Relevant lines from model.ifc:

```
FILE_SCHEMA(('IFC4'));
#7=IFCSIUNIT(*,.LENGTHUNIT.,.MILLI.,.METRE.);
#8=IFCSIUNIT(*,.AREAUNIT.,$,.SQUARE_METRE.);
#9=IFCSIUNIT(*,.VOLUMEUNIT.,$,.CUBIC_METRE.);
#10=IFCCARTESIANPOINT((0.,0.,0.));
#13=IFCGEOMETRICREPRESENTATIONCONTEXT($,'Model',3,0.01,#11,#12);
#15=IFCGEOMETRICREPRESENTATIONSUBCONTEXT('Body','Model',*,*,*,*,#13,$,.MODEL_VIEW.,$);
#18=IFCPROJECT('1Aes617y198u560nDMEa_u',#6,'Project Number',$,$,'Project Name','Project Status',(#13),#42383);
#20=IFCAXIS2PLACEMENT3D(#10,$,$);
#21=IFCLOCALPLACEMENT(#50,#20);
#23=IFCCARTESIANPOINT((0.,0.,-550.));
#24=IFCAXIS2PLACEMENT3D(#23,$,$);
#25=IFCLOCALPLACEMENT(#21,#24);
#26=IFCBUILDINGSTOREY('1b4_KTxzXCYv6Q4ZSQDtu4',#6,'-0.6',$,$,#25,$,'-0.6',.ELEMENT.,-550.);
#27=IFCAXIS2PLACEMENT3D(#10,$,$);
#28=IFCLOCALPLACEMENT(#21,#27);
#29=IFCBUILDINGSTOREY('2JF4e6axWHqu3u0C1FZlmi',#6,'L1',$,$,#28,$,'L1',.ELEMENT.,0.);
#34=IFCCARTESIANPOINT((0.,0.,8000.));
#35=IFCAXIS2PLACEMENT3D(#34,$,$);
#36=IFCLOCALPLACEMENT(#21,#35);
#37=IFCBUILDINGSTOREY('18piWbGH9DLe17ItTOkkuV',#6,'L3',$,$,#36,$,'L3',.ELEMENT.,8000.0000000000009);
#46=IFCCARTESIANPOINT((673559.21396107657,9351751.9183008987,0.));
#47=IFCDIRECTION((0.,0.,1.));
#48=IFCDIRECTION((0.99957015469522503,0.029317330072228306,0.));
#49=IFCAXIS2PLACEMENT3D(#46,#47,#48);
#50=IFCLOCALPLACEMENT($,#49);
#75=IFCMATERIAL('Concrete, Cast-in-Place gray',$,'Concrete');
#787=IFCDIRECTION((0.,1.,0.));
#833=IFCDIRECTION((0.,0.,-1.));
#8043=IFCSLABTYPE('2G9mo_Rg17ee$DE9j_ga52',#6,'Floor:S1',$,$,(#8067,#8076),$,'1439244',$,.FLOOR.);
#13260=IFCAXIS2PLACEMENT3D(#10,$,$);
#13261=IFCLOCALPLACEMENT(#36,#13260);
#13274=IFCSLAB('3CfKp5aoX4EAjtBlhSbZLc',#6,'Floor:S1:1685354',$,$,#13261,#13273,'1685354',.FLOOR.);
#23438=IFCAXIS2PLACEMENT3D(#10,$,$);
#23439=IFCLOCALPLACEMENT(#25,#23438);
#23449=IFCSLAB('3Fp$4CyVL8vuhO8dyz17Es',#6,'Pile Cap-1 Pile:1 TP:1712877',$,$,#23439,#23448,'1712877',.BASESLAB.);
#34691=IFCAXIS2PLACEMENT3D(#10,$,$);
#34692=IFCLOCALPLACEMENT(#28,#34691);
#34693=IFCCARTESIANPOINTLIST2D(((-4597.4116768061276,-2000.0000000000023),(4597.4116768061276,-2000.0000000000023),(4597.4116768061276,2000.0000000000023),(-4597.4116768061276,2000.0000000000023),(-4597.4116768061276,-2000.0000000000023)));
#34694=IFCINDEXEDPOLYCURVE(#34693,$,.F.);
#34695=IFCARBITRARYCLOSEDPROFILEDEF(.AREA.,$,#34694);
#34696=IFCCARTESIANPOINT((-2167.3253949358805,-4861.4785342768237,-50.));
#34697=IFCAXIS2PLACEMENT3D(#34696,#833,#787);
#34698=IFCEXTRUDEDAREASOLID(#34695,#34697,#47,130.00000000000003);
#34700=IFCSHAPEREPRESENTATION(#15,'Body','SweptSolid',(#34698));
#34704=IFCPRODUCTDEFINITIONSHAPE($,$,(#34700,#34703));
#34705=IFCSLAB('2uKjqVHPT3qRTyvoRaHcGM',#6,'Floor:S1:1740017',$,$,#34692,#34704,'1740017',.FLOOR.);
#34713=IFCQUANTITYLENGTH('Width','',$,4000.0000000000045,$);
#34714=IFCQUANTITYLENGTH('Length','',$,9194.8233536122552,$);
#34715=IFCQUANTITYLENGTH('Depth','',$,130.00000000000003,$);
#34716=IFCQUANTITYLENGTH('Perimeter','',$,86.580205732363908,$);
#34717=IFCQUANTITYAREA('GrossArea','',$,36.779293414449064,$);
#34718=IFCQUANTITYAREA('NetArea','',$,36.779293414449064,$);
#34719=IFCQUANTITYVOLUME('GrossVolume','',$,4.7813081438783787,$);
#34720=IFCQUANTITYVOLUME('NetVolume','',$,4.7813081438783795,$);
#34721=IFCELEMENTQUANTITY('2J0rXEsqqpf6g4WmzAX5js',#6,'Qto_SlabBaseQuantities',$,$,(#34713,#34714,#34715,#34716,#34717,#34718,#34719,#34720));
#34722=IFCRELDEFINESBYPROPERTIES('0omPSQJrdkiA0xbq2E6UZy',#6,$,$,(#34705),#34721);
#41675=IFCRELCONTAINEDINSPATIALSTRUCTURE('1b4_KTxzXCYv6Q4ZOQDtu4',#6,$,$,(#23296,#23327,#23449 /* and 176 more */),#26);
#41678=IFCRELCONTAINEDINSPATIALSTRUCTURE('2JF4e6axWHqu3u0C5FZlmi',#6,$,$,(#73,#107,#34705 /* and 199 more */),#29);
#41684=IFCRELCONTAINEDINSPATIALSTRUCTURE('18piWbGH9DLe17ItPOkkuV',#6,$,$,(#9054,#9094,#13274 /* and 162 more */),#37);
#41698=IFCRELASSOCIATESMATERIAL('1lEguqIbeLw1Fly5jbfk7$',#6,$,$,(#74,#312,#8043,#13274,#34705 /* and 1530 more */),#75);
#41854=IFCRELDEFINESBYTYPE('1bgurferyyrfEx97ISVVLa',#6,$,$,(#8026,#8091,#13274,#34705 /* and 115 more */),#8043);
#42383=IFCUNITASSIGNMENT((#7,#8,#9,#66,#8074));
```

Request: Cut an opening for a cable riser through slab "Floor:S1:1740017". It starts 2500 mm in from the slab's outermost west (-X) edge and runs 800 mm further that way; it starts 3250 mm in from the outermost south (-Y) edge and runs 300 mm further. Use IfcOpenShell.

```python
import numpy as np
import ifcopenshell
import ifcopenshell.api.feature
import ifcopenshell.api.geometry
import ifcopenshell.api.pset
import ifcopenshell.api.root
import ifcopenshell.geom
import ifcopenshell.util.element
import ifcopenshell.util.placement
import ifcopenshell.util.representation
import ifcopenshell.util.shape
import ifcopenshell.util.unit

model = ifcopenshell.open("model.ifc")
unit_scale = ifcopenshell.util.unit.calculate_unit_scale(model)
area_scale = ifcopenshell.util.unit.calculate_unit_scale(model, "AREAUNIT")
volume_scale = ifcopenshell.util.unit.calculate_unit_scale(model, "VOLUMEUNIT")
settings = ifcopenshell.geom.settings()


def volume(element):
    """Net volume in cubic metres, openings subtracted."""
    shape = ifcopenshell.geom.create_shape(settings, element)
    return ifcopenshell.util.shape.get_volume(shape.geometry)


slab = model.by_guid("2uKjqVHPT3qRTyvoRaHcGM")
before = volume(slab)

# Extent in the slab's own axes, in metres. The edges named are its -X and -Y sides.
slab_shape = ifcopenshell.geom.create_shape(settings, slab)
vertices = ifcopenshell.util.shape.get_vertices(slab_shape.geometry)
x_min, y_min, bottom = vertices.min(axis=0)
top = vertices[:, 2].max()

opening = ifcopenshell.api.root.create_entity(model, ifc_class="IfcOpeningElement", name="Cable riser opening", predefined_type="OPENING")
context = ifcopenshell.util.representation.get_context(model, "Model", "Body", "MODEL_VIEW")
width, depth = 0.8, 0.3
outline = [(0.0, 0.0), (width, 0.0), (width, depth), (0.0, depth), (0.0, 0.0)]
# Overshoot both faces by 50 mm so the cut is clean.
shape = ifcopenshell.api.geometry.add_slab_representation(
    model, context=context, depth=top - bottom + 0.1, polyline=outline
)
ifcopenshell.api.geometry.assign_representation(model, product=opening, representation=shape)

matrix = ifcopenshell.util.placement.get_local_placement(slab.ObjectPlacement)
matrix[:, 3] = matrix @ np.append(np.array([x_min + 2.5, y_min + 3.25, bottom - 0.05]) / unit_scale, 1.0)
ifcopenshell.api.geometry.edit_object_placement(model, product=opening, matrix=matrix, is_si=False)
ifcopenshell.api.feature.add_feature(model, feature=opening, element=slab)

after = volume(slab)

# Update the slab's stored quantities.
qto = model.by_id(ifcopenshell.util.element.get_pset(slab, "Qto_SlabBaseQuantities", should_inherit=False)["id"])
ifcopenshell.api.pset.edit_qto(model, qto=qto, properties={
    "NetArea": after / (top - bottom) / area_scale,
    "NetVolume": after / volume_scale,
})

print(f"slab volume {before:.3f} -> {after:.3f} m3")

model.write("model_edited.ifc")
```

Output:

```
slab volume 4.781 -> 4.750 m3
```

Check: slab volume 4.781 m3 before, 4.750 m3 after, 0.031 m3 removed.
